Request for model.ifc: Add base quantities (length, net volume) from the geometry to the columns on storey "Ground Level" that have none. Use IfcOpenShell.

First a look at what the model holds.

```python
import ifcopenshell
import ifcopenshell.util.element
import ifcopenshell.util.unit

model = ifcopenshell.open("model.ifc")
print(model.schema)
for unit_type in ("LENGTHUNIT", "AREAUNIT", "VOLUMEUNIT"):
    print(unit_type, ifcopenshell.util.unit.calculate_unit_scale(model, unit_type))
storey = next(s for s in model.by_type("IfcBuildingStorey") if s.Name == "Ground Level")
columns = [e for e in ifcopenshell.util.element.get_decomposition(storey) if e.is_a("IfcColumn")]
for e in sorted(columns, key=lambda e: e.id()):
    print(e.id(), e.is_a(), e.Name, list(ifcopenshell.util.element.get_psets(e, qtos_only=True)), sep=" | ")
```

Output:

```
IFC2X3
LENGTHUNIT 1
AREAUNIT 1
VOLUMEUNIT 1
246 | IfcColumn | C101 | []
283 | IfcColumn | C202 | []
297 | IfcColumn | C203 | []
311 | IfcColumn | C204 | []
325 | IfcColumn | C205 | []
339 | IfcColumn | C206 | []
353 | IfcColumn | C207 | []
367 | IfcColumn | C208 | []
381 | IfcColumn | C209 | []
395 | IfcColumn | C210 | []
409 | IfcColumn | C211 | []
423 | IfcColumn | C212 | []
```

```python
import ifcopenshell
import ifcopenshell.api.pset
import ifcopenshell.geom
import ifcopenshell.util.element
import ifcopenshell.util.shape
import ifcopenshell.util.unit

model = ifcopenshell.open("model.ifc")
unit_scale = ifcopenshell.util.unit.calculate_unit_scale(model)
volume_scale = ifcopenshell.util.unit.calculate_unit_scale(model, "VOLUMEUNIT")
settings = ifcopenshell.geom.settings()

storey = next(s for s in model.by_type("IfcBuildingStorey") if s.Name == "Ground Level")
columns = [e for e in ifcopenshell.util.element.get_decomposition(storey) if e.is_a("IfcColumn")]

for e in sorted(columns, key=lambda e: e.id()):
    if ifcopenshell.util.element.get_psets(e, qtos_only=True, should_inherit=False):
        continue
    # Geometry comes back in metres, in the element's own axes.
    shape = ifcopenshell.geom.create_shape(settings, e)
    values = {
        "Length": ifcopenshell.util.shape.get_z(shape.geometry) / unit_scale,
        "NetVolume": ifcopenshell.util.shape.get_volume(shape.geometry) / volume_scale,
    }
    qto = ifcopenshell.api.pset.add_qto(model, product=e, name="BaseQuantities")
    ifcopenshell.api.pset.edit_qto(model, qto=qto, properties=values)
    print(e.id(), {k: round(v, 3) for k, v in values.items()})

model.write("model_v2.ifc")
```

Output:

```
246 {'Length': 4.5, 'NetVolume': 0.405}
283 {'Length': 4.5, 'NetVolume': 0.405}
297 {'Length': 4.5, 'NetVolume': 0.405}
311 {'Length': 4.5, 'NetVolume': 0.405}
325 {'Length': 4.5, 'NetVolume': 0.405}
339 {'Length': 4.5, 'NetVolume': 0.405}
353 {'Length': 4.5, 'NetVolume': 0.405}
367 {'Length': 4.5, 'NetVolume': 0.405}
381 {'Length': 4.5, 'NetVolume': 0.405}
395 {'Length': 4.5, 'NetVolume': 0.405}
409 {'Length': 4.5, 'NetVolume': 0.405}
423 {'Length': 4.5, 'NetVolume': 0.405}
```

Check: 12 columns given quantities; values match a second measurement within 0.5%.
